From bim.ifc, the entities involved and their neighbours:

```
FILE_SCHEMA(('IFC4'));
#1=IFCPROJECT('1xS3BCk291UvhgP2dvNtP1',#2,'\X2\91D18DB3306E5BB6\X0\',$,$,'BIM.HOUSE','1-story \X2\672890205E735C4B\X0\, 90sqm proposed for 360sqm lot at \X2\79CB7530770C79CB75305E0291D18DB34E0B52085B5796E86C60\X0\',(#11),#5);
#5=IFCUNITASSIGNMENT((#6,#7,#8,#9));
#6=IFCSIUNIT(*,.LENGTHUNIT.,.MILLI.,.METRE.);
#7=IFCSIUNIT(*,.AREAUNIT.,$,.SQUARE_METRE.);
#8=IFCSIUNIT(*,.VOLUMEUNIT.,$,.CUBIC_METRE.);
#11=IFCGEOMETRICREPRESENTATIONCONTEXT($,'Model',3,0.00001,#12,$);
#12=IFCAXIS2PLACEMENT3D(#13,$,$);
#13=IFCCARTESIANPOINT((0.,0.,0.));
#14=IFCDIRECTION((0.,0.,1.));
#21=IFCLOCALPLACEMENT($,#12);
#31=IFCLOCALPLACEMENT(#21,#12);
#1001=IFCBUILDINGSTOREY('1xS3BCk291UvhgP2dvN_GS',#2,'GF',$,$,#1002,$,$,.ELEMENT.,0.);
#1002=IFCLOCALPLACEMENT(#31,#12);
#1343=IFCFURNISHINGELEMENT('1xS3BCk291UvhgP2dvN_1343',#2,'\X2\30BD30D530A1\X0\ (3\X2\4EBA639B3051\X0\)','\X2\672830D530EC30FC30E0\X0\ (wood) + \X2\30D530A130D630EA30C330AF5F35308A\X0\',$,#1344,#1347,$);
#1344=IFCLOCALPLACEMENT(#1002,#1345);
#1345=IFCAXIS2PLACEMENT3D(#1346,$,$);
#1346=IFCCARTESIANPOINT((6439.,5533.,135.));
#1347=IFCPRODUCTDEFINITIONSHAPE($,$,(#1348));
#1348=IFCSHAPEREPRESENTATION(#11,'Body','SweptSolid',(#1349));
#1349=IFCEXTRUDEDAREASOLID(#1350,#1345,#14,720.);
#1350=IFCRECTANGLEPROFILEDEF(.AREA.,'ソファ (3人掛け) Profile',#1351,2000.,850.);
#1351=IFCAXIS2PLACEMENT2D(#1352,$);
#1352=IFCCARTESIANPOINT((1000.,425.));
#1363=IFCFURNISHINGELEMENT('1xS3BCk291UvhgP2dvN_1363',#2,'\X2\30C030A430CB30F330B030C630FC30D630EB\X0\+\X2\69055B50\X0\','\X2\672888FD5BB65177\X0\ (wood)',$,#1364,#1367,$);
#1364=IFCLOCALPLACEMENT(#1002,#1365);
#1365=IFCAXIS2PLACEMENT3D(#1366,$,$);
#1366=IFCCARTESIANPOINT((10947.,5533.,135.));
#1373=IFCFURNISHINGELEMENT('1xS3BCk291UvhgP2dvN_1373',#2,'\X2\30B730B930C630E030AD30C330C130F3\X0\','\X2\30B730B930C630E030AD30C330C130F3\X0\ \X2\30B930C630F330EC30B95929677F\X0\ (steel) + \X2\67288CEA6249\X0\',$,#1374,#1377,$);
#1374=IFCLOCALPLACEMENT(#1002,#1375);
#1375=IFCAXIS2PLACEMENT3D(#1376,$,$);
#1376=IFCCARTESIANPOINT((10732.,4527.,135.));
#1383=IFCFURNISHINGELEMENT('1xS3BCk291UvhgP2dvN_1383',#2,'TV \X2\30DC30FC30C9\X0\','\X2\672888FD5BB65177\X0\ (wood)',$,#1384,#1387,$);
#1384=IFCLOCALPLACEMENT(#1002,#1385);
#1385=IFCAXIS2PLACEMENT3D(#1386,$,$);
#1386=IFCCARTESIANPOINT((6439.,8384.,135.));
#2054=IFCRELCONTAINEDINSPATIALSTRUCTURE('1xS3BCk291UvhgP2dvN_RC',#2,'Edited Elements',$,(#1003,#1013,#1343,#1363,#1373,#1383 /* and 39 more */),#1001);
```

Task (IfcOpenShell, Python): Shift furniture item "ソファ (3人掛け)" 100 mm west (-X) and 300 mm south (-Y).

```python
import ifcopenshell
import ifcopenshell.api.geometry
import ifcopenshell.util.placement

model = ifcopenshell.open("bim.ifc")

item = model.by_guid("1xS3BCk291UvhgP2dvN_1343")
matrix = ifcopenshell.util.placement.get_local_placement(item.ObjectPlacement)
matrix[0, 3] -= 100.0
matrix[1, 3] -= 300.0
ifcopenshell.api.geometry.edit_object_placement(model, product=item, matrix=matrix, is_si=False)

print(ifcopenshell.util.placement.get_local_placement(item.ObjectPlacement).round(3) + 0.0)

model.write("bim_updated.ifc")
```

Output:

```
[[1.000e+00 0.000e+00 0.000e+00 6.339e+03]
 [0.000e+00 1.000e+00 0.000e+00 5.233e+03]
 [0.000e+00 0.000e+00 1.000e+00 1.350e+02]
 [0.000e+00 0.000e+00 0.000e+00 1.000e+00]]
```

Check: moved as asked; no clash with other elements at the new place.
